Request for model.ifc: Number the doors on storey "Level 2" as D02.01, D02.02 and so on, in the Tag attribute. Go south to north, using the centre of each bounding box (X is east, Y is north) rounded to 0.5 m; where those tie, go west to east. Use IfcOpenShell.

First a look at what the model holds.

```python
import ifcopenshell
import ifcopenshell.util.element
import ifcopenshell.util.placement

model = ifcopenshell.open("model.ifc")
print(model.schema)
storey = next(s for s in model.by_type("IfcBuildingStorey") if s.Name == "Level 2")
doors = [e for e in ifcopenshell.util.element.get_decomposition(storey) if e.is_a("IfcDoor")]
for e in sorted(doors, key=lambda e: e.id()):
    origin = ifcopenshell.util.placement.get_local_placement(e.ObjectPlacement)[:3, 3]
    print(e.id(), e.Tag, e.Name, origin.round(2) + 0.0, sep=" | ")
```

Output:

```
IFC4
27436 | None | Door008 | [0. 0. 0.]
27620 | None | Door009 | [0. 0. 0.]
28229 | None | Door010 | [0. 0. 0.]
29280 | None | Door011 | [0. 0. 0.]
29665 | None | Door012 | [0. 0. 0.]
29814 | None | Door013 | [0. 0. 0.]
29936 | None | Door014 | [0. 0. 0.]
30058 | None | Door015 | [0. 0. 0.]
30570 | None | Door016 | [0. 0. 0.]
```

```python
import ifcopenshell
import ifcopenshell.geom
import ifcopenshell.util.element
import ifcopenshell.util.shape

model = ifcopenshell.open("model.ifc")
settings = ifcopenshell.geom.settings()
settings.set("use-world-coords", True)


def centre(element):
    shape = ifcopenshell.geom.create_shape(settings, element)
    return ifcopenshell.util.shape.get_bbox_centroid(shape.geometry)


storey = next(s for s in model.by_type("IfcBuildingStorey") if s.Name == "Level 2")
doors = [e for e in ifcopenshell.util.element.get_decomposition(storey) if e.is_a("IfcDoor")]

# Insertion points can sit at a corner or the storey origin, so sort by the geometry (in metres).
centres = {e: centre(e) for e in doors}
doors.sort(key=lambda e: (round(centres[e][1] / 0.5), centres[e][0]))

for i, e in enumerate(doors, start=1):
    number = f"D02.{i:02d}"
    e.Tag = number
    print(e.id(), number)

model.write("model_updated.ifc")
```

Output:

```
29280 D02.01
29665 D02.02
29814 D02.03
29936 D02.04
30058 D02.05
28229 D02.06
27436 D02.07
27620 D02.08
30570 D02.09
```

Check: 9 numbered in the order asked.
